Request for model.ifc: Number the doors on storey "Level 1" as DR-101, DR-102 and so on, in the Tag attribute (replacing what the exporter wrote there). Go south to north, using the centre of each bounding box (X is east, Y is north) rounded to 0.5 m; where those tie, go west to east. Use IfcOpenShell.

First a look at what the model holds.

```python
import ifcopenshell
import ifcopenshell.util.element
import ifcopenshell.util.placement

model = ifcopenshell.open("model.ifc")
print(model.schema)
storey = next(s for s in model.by_type("IfcBuildingStorey") if s.Name == "Level 1")
doors = [e for e in ifcopenshell.util.element.get_decomposition(storey) if e.is_a("IfcDoor")]
for e in sorted(doors, key=lambda e: e.id()):
    origin = ifcopenshell.util.placement.get_local_placement(e.ObjectPlacement)[:3, 3]
    print(e.id(), e.Tag, e.Name, origin.round(2) + 0.0, sep=" | ")
```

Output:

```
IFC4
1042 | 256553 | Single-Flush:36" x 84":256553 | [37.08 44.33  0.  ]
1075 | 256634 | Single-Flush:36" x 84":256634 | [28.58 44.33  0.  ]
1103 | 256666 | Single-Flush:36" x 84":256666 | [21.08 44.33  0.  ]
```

```python
import ifcopenshell
import ifcopenshell.geom
import ifcopenshell.util.element
import ifcopenshell.util.shape

model = ifcopenshell.open("model.ifc")
settings = ifcopenshell.geom.settings()
settings.set("use-world-coords", True)


def centre(element):
    shape = ifcopenshell.geom.create_shape(settings, element)
    return ifcopenshell.util.shape.get_bbox_centroid(shape.geometry)


storey = next(s for s in model.by_type("IfcBuildingStorey") if s.Name == "Level 1")
doors = [e for e in ifcopenshell.util.element.get_decomposition(storey) if e.is_a("IfcDoor")]

# Insertion points can sit at a corner or the storey origin, so sort by the geometry (in metres).
centres = {e: centre(e) for e in doors}
doors.sort(key=lambda e: (round(centres[e][1] / 0.5), centres[e][0]))

for i, e in enumerate(doors, start=1):
    number = f"DR-1{i:02d}"
    e.Tag = number
    print(e.id(), number)

model.write("model-out.ifc")
```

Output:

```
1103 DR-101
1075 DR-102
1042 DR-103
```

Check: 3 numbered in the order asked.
